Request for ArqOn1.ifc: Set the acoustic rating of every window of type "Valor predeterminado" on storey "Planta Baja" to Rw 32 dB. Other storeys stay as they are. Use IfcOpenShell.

First a look at what the model holds.

```python
import ifcopenshell
import ifcopenshell.util.element

model = ifcopenshell.open("ArqOn1.ifc")
print(model.schema)
storey = next(s for s in model.by_type("IfcBuildingStorey") if s.Name == "Planta Baja")
windows = [e for e in ifcopenshell.util.element.get_decomposition(storey) if e.is_a("IfcWindow")]
seen = {}
for e in windows:
    element_type = ifcopenshell.util.element.get_type(e)
    key = (element_type.Name if element_type != e and element_type else None, ifcopenshell.util.element.get_pset(e, "Pset_WindowCommon", "AcousticRating"))
    seen[key] = seen.get(key, 0) + 1
for (name, value), count in sorted(seen.items(), key=str):
    print(count, "x", name, "|", value)
```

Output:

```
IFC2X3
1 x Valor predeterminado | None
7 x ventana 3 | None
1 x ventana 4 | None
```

```python
import ifcopenshell
import ifcopenshell.api.pset
import ifcopenshell.util.element

model = ifcopenshell.open("ArqOn1.ifc")

storey = next(s for s in model.by_type("IfcBuildingStorey") if s.Name == "Planta Baja")
windows = [e for e in ifcopenshell.util.element.get_decomposition(storey) if e.is_a("IfcWindow")]

count = 0
for e in windows:
    element_type = ifcopenshell.util.element.get_type(e)
    if element_type in (None, e) or element_type.Name != "Valor predeterminado":
        continue
    # add_pset returns the element's existing set when there is one.
    pset = ifcopenshell.api.pset.add_pset(model, product=e, name="Pset_WindowCommon")
    ifcopenshell.api.pset.edit_pset(model, pset=pset, properties={"AcousticRating": "Rw 32 dB"})
    count += 1

print(count, "windows updated")

model.write("ArqOn1_edited.ifc")
```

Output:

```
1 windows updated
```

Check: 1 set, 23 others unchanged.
